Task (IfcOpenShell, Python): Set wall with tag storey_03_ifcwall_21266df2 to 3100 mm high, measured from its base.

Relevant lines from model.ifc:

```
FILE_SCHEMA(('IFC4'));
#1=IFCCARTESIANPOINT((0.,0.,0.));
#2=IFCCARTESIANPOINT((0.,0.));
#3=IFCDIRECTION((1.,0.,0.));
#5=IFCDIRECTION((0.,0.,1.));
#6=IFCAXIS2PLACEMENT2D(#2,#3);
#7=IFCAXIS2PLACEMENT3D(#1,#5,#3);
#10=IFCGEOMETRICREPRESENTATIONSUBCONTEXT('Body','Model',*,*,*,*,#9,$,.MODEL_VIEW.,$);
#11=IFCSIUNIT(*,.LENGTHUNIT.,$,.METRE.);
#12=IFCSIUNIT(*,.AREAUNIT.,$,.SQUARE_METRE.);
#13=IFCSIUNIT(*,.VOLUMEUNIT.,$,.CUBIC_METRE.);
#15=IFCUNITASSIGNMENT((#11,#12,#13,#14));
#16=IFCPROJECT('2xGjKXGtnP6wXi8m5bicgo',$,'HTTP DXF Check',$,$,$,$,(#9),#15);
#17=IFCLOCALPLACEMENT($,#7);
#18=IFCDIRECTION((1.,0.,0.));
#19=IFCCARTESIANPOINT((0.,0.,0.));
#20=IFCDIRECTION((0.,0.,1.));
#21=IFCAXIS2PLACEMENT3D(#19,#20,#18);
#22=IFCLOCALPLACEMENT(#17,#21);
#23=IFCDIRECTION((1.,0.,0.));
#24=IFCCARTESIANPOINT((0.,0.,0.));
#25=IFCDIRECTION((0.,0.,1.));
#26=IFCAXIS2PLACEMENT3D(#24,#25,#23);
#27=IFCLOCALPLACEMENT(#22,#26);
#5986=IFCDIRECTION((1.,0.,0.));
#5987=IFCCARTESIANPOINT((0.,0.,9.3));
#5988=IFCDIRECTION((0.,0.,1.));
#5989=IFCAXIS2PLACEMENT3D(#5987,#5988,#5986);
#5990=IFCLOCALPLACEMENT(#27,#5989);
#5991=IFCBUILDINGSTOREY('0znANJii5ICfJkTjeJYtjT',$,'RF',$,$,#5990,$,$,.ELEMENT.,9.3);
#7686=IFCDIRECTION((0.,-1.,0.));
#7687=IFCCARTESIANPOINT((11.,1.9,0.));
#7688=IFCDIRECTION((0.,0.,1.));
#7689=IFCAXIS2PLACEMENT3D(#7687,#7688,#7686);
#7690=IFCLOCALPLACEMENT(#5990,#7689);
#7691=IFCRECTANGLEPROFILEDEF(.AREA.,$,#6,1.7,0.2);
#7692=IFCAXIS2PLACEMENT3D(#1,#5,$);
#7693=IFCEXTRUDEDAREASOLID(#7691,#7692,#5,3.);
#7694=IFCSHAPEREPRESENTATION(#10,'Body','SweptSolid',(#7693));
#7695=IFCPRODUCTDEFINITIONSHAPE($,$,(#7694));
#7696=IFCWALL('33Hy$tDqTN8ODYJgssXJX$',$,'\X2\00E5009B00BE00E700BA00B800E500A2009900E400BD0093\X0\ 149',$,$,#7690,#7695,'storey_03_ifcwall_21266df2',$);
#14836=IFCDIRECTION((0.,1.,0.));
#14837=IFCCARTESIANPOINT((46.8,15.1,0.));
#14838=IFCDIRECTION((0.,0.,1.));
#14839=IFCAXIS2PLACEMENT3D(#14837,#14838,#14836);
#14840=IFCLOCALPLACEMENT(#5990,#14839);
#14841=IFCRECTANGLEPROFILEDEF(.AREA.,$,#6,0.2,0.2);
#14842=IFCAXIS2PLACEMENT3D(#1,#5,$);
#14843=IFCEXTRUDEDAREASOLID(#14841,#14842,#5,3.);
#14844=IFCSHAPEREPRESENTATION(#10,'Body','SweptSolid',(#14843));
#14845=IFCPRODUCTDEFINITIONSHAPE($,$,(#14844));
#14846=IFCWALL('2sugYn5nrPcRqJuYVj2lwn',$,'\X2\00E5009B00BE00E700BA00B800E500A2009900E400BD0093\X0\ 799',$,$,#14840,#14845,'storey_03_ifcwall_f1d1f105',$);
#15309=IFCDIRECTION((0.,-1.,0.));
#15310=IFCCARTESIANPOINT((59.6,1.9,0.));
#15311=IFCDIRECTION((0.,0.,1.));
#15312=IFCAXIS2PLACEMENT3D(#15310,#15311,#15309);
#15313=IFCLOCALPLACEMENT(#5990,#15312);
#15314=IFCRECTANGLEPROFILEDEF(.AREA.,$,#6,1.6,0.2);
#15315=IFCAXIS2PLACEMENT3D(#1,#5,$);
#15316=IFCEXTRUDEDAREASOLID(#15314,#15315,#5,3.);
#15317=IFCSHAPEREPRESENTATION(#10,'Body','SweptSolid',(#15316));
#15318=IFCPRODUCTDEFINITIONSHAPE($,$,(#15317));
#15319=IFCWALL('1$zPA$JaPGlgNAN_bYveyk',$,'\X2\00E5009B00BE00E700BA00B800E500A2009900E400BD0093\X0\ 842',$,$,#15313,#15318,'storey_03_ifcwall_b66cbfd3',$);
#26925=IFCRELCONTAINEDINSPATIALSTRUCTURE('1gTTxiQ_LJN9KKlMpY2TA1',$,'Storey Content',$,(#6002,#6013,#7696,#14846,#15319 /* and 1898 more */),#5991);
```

```python
import ifcopenshell
import ifcopenshell.geom
import ifcopenshell.util.representation
import ifcopenshell.util.shape
import ifcopenshell.util.unit

model = ifcopenshell.open("model.ifc")
unit_scale = ifcopenshell.util.unit.calculate_unit_scale(model)
settings = ifcopenshell.geom.settings()


def volume(element):
    """Net volume in cubic metres, openings subtracted."""
    shape = ifcopenshell.geom.create_shape(settings, element)
    return ifcopenshell.util.shape.get_volume(shape.geometry)


wall = model.by_guid("33Hy$tDqTN8ODYJgssXJX$")
before = volume(wall)

body = ifcopenshell.util.representation.get_representation(wall, "Model", "Body")
solid = body.Items[0]
old_height = solid.Depth
solid.Depth = 3.1 / unit_scale
after = volume(wall)

print(f"height {old_height:g} -> {solid.Depth:g}, volume {before:.3f} -> {after:.3f} m3")

model.write("model_updated.ifc")
```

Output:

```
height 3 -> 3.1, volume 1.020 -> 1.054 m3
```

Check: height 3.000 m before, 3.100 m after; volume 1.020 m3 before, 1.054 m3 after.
